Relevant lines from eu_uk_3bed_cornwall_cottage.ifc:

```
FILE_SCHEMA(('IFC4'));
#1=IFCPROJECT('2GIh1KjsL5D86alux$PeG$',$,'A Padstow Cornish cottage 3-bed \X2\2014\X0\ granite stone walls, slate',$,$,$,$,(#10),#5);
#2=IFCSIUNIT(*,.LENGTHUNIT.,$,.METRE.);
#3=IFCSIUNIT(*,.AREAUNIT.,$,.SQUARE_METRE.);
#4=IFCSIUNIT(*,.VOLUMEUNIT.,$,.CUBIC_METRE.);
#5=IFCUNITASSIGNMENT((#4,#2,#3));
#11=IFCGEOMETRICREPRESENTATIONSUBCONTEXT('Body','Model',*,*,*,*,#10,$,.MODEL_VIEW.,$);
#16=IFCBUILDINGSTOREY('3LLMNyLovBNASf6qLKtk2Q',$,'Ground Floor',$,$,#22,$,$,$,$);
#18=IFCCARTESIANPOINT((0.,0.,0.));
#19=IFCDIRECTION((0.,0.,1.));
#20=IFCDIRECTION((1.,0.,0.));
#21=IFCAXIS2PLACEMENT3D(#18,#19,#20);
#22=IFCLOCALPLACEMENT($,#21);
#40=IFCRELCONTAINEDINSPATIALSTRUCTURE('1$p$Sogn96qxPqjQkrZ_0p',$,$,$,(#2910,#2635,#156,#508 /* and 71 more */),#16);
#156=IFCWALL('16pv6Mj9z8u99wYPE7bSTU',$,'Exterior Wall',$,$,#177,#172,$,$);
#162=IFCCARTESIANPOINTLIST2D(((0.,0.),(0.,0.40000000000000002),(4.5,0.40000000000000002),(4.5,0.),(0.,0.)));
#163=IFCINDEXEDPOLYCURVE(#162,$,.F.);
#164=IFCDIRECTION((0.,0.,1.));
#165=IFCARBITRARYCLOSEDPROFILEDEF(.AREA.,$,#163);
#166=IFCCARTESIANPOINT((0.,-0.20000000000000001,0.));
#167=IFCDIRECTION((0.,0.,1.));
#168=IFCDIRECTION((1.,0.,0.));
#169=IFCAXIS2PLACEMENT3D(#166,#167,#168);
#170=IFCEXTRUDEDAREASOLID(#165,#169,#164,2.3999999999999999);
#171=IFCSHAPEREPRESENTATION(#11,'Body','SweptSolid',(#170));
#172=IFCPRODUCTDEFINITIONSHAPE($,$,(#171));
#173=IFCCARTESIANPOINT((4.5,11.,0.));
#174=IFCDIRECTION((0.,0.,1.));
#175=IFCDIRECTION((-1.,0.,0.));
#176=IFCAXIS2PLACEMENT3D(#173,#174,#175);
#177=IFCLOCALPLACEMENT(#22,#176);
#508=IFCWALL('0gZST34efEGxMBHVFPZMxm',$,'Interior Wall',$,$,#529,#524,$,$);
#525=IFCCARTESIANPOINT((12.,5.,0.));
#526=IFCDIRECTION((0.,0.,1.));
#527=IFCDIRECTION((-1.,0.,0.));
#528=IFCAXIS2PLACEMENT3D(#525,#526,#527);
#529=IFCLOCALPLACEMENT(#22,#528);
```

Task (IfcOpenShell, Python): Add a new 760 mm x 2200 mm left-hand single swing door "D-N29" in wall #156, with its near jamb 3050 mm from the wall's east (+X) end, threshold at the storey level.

```python
import numpy as np
import ifcopenshell
import ifcopenshell.api.feature
import ifcopenshell.api.geometry
import ifcopenshell.api.root
import ifcopenshell.api.spatial
import ifcopenshell.geom
import ifcopenshell.util.element
import ifcopenshell.util.placement
import ifcopenshell.util.representation
import ifcopenshell.util.shape
import ifcopenshell.util.unit

model = ifcopenshell.open("eu_uk_3bed_cornwall_cottage.ifc")
unit_scale = ifcopenshell.util.unit.calculate_unit_scale(model)
settings = ifcopenshell.geom.settings()


def volume(element):
    """Net volume in cubic metres, openings subtracted."""
    shape = ifcopenshell.geom.create_shape(settings, element)
    return ifcopenshell.util.shape.get_volume(shape.geometry)


wall = model.by_guid("16pv6Mj9z8u99wYPE7bSTU")
storey = ifcopenshell.util.element.get_container(wall, ifc_class="IfcBuildingStorey")
context = ifcopenshell.util.representation.get_context(model, "Model", "Body", "MODEL_VIEW")
before = volume(wall)

width, height, from_end, sill = 0.76, 2.2, 3.05, 0.0  # metres

# The wall runs along its own X axis, and the end named is its -X end.
wall_shape = ifcopenshell.geom.create_shape(settings, wall)
x, y, z = ifcopenshell.util.shape.get_vertices(wall_shape.geometry).T
start = x.min() + from_end
face, thickness = float(y.min()), float(y.max() - y.min())
wall_matrix = ifcopenshell.util.placement.get_local_placement(wall.ObjectPlacement)
level = ifcopenshell.util.placement.get_local_placement(storey.ObjectPlacement)[2, 3]


def in_wall(x, y):
    """Placement at x, y metres in the wall's axes, at sill height."""
    matrix = wall_matrix.copy()
    matrix[:, 3] = wall_matrix @ np.array([x / unit_scale, y / unit_scale, 0.0, 1.0])
    matrix[2, 3] = level + sill / unit_scale
    return matrix


# Opening: a box that overshoots both wall faces by 50 mm.
opening = ifcopenshell.api.root.create_entity(model, ifc_class="IfcOpeningElement", predefined_type="OPENING")
box = ifcopenshell.api.geometry.add_wall_representation(
    model, context=context, length=width, height=height, thickness=thickness + 0.1
)
ifcopenshell.api.geometry.assign_representation(model, product=opening, representation=box)
ifcopenshell.api.geometry.edit_object_placement(model, product=opening, matrix=in_wall(start, face - 0.05), is_si=False)
ifcopenshell.api.feature.add_feature(model, feature=opening, element=wall)

door = ifcopenshell.api.root.create_entity(model, ifc_class="IfcDoor", name="D-N29", predefined_type="DOOR")
door.OverallWidth, door.OverallHeight = width / unit_scale, height / unit_scale
door.OperationType = "SINGLE_SWING_LEFT"
body = ifcopenshell.api.geometry.add_door_representation(
    model,
    context=context,
    overall_width=door.OverallWidth,
    overall_height=door.OverallHeight,
    operation_type="SINGLE_SWING_LEFT",
    lining_properties={"LiningDepth": thickness / unit_scale, "ThresholdDepth": thickness / unit_scale},
)
ifcopenshell.api.geometry.assign_representation(model, product=door, representation=body)
ifcopenshell.api.spatial.assign_container(model, products=[door], relating_structure=storey)
ifcopenshell.api.feature.add_filling(model, opening=opening, element=door)

# The lining spans the wall, so the door starts at the wall face.
ifcopenshell.api.geometry.edit_object_placement(model, product=door, matrix=in_wall(start, face), is_si=False)

after = volume(wall)

print(f"wall volume {before:.3f} -> {after:.3f} m3")

model.write("eu_uk_3bed_cornwall_cottage_edited.ifc")
```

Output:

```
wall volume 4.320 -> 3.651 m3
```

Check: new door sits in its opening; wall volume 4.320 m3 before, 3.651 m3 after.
